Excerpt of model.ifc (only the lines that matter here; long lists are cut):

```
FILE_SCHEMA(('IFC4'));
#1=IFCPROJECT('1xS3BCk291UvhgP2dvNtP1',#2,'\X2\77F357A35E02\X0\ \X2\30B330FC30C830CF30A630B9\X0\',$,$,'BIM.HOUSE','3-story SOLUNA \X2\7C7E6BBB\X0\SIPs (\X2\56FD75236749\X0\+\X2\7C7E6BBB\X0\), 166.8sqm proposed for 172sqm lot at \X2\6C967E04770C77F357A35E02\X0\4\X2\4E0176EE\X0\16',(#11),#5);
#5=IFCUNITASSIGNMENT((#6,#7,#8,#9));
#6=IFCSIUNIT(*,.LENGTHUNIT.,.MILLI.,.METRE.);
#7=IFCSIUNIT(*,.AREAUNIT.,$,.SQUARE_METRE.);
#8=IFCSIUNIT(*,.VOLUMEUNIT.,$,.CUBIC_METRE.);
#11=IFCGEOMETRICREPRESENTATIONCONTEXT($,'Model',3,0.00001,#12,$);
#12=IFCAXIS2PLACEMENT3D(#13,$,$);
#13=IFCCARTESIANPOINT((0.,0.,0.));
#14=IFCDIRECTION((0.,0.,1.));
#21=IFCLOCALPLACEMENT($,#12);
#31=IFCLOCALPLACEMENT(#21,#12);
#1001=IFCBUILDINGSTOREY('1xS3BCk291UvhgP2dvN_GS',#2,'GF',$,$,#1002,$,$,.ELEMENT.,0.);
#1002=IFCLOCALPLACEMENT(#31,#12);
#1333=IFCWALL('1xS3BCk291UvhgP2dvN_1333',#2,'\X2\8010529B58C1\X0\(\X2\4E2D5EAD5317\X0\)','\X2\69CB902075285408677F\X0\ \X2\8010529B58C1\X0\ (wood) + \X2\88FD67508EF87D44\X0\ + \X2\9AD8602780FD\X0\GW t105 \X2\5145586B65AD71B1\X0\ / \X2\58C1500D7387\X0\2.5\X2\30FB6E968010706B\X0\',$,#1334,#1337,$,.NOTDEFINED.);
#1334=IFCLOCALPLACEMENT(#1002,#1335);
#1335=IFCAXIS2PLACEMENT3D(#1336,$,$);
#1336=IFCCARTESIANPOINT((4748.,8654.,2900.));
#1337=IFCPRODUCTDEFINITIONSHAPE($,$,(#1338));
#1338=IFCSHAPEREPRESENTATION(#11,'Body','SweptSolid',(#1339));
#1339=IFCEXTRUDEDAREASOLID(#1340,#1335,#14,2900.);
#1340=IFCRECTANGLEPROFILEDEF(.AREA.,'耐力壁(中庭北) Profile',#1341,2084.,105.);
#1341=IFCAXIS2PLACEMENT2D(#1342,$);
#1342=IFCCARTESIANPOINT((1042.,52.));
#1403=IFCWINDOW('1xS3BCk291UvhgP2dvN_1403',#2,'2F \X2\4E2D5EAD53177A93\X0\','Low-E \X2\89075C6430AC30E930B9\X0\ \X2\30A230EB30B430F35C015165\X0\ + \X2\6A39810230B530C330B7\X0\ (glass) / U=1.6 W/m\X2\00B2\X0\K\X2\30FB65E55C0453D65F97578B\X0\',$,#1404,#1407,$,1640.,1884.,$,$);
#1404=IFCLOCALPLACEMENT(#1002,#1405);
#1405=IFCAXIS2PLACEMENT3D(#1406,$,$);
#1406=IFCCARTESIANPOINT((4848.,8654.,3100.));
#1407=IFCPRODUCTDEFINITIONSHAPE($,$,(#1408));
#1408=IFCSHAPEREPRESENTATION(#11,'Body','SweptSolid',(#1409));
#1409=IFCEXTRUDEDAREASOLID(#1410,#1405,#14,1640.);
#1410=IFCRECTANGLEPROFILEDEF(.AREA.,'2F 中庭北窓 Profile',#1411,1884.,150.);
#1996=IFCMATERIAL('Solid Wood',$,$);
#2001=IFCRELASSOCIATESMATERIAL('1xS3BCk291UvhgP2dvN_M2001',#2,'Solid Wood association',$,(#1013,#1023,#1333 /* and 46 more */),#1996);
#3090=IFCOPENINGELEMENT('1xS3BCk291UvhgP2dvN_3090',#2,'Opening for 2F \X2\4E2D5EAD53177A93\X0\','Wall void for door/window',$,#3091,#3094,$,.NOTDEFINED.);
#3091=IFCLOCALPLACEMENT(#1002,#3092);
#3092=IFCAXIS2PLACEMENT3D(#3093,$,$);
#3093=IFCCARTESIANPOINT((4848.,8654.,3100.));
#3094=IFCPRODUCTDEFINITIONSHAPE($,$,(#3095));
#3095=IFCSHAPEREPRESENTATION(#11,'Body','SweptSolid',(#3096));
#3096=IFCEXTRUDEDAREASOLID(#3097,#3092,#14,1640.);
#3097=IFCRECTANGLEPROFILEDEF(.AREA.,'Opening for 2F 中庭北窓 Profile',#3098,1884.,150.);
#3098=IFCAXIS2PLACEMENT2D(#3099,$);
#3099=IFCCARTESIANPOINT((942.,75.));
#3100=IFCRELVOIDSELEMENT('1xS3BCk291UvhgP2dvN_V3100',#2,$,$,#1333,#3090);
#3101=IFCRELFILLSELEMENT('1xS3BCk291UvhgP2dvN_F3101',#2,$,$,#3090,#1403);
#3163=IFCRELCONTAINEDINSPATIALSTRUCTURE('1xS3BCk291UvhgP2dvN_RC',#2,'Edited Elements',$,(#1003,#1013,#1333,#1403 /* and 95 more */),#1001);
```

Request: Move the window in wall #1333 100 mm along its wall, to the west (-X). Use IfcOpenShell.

```python
import ifcopenshell
import ifcopenshell.api.geometry
import ifcopenshell.util.placement

model = ifcopenshell.open("model.ifc")

window = model.by_id(1403)
opening = window.FillsVoids[0].RelatingOpeningElement
wall = opening.VoidsElements[0].RelatingBuildingElement

wall_matrix = ifcopenshell.util.placement.get_local_placement(wall.ObjectPlacement)
shift = wall_matrix[:3, 0] * -100.0
before = ifcopenshell.util.placement.get_local_placement(window.ObjectPlacement)[:3, 3].copy()

# The window is not placed relative to its opening, so move both.
for product in (opening, window):
    matrix = ifcopenshell.util.placement.get_local_placement(product.ObjectPlacement)
    matrix[:3, 3] += shift
    ifcopenshell.api.geometry.edit_object_placement(model, product=product, matrix=matrix, is_si=False)

after = ifcopenshell.util.placement.get_local_placement(window.ObjectPlacement)[:3, 3]
print("window moved by", (after - before).round(3) + 0.0)

model.write("model_v2.ifc")
```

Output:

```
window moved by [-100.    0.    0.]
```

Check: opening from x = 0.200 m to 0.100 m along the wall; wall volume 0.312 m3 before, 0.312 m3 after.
